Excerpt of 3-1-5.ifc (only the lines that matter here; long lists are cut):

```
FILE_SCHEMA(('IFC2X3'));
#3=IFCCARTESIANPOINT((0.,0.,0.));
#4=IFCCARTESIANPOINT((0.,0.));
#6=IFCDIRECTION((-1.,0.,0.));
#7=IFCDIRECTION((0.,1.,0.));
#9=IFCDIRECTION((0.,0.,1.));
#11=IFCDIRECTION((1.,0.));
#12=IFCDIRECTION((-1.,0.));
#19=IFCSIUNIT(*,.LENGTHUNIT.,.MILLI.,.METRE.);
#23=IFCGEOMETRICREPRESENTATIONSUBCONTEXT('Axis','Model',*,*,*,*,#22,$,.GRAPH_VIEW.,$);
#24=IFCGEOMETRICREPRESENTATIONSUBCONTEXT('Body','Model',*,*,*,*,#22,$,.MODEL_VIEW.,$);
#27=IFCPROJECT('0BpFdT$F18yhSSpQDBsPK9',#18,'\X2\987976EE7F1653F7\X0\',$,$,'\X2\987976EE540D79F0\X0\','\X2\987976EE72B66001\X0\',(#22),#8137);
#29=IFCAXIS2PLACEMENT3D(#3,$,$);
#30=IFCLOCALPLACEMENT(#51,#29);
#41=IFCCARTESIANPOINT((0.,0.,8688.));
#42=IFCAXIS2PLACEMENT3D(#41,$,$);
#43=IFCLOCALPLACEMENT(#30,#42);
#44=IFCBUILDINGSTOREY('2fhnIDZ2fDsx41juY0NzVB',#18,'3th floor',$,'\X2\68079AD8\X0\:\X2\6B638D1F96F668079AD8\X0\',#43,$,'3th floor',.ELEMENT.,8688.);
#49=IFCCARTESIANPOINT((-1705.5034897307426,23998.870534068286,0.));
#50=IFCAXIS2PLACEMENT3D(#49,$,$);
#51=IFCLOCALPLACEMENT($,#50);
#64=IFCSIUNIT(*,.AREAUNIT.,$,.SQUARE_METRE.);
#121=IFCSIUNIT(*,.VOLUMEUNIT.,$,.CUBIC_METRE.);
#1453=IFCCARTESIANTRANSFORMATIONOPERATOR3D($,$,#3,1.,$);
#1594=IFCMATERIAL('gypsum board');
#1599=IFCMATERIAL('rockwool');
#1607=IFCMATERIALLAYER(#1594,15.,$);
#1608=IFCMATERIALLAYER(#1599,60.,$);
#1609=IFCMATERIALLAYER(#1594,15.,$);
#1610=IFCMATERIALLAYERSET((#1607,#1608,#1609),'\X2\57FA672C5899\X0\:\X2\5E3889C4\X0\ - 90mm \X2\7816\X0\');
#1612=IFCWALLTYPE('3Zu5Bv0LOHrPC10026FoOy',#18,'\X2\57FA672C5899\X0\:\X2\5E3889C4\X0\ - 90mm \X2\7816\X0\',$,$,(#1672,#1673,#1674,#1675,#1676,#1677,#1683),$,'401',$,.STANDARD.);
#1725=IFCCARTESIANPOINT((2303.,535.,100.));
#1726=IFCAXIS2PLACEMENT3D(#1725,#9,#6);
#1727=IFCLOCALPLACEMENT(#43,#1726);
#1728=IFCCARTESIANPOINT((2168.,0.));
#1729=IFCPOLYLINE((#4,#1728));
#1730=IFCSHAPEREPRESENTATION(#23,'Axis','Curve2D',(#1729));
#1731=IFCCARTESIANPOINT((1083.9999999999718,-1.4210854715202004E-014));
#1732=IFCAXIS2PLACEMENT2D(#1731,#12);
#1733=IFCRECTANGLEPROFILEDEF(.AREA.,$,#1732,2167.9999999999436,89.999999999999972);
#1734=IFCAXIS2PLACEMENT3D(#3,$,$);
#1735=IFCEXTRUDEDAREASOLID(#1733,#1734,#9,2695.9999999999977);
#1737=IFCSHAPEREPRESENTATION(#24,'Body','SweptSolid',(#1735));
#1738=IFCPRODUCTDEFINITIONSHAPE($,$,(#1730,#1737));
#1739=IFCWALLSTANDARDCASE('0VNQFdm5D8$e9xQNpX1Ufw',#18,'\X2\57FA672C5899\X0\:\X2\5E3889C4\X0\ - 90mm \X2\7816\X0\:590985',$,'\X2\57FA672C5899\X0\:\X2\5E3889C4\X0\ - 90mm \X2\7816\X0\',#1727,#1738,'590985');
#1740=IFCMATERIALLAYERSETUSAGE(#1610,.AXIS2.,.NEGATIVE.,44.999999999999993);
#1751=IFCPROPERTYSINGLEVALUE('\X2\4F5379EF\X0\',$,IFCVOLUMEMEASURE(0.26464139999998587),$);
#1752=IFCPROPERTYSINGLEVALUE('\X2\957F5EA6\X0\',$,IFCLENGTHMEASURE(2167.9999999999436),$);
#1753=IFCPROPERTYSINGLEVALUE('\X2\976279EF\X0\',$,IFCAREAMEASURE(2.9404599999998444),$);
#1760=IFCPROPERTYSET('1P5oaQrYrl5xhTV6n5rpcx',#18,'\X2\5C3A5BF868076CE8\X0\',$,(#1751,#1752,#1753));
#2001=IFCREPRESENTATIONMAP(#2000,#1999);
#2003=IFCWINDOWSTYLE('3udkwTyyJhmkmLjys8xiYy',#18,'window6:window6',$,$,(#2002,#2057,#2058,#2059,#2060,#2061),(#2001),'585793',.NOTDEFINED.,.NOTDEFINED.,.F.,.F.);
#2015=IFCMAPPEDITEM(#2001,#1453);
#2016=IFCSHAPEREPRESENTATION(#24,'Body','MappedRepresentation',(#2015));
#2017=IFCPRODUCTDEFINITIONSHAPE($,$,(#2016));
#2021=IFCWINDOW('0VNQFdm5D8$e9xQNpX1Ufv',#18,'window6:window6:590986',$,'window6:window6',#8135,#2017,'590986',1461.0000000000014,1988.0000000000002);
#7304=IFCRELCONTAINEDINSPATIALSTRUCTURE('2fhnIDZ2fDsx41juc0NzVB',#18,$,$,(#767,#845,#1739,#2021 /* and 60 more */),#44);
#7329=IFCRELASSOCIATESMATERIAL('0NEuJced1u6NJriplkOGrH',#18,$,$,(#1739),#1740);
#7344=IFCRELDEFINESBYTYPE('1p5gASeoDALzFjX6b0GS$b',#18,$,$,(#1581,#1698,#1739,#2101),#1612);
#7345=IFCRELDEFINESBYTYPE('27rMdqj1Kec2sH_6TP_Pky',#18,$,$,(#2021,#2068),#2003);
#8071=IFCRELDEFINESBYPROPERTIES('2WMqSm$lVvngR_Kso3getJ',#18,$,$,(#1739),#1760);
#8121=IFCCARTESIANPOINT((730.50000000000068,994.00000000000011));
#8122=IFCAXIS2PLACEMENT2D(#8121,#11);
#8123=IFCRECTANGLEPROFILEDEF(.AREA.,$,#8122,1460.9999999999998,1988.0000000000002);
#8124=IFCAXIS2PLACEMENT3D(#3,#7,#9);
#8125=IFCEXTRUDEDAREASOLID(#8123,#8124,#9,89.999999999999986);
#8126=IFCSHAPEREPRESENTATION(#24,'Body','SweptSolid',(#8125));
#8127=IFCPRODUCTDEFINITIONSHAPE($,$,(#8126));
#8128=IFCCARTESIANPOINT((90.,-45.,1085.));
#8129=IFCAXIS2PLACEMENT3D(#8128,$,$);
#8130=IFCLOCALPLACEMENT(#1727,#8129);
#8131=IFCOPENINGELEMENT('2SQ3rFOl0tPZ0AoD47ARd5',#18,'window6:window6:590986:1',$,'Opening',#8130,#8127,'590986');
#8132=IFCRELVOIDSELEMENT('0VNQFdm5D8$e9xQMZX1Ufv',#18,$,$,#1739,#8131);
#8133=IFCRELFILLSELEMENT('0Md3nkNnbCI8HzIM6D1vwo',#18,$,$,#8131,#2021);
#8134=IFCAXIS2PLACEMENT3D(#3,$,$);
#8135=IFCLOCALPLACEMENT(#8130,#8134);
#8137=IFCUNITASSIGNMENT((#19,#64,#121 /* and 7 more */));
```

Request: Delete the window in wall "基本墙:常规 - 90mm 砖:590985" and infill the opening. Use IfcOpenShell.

```python
import ifcopenshell
import ifcopenshell.api.feature
import ifcopenshell.api.pset
import ifcopenshell.api.root
import ifcopenshell.geom
import ifcopenshell.util.element
import ifcopenshell.util.shape
import ifcopenshell.util.unit

model = ifcopenshell.open("3-1-5.ifc")
area_scale = ifcopenshell.util.unit.calculate_unit_scale(model, "AREAUNIT")
volume_scale = ifcopenshell.util.unit.calculate_unit_scale(model, "VOLUMEUNIT")
settings = ifcopenshell.geom.settings()


def volume(element):
    """Net volume in cubic metres, openings subtracted."""
    shape = ifcopenshell.geom.create_shape(settings, element)
    return ifcopenshell.util.shape.get_volume(shape.geometry)


window = model.by_guid("0VNQFdm5D8$e9xQNpX1Ufv")
opening = window.FillsVoids[0].RelatingOpeningElement
wall = opening.VoidsElements[0].RelatingBuildingElement
before = volume(wall)

ifcopenshell.api.root.remove_product(model, product=window)
ifcopenshell.api.feature.remove_feature(model, feature=opening)

after = volume(wall)
thickness = 0.09  # wall thickness in metres

# Update the wall's stored quantities.
pset = model.by_id(ifcopenshell.util.element.get_pset(wall, "尺寸标注", should_inherit=False)["id"])
ifcopenshell.api.pset.edit_pset(model, pset=pset, properties={
    "体积": model.create_entity("IfcVolumeMeasure", after / volume_scale),
    "面积": model.create_entity("IfcAreaMeasure", after / thickness / area_scale),
})

print(f"wall volume {before:.3f} -> {after:.3f} m3")

model.write("3-1-5-out.ifc")
```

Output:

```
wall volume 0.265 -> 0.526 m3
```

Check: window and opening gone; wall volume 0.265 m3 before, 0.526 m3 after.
